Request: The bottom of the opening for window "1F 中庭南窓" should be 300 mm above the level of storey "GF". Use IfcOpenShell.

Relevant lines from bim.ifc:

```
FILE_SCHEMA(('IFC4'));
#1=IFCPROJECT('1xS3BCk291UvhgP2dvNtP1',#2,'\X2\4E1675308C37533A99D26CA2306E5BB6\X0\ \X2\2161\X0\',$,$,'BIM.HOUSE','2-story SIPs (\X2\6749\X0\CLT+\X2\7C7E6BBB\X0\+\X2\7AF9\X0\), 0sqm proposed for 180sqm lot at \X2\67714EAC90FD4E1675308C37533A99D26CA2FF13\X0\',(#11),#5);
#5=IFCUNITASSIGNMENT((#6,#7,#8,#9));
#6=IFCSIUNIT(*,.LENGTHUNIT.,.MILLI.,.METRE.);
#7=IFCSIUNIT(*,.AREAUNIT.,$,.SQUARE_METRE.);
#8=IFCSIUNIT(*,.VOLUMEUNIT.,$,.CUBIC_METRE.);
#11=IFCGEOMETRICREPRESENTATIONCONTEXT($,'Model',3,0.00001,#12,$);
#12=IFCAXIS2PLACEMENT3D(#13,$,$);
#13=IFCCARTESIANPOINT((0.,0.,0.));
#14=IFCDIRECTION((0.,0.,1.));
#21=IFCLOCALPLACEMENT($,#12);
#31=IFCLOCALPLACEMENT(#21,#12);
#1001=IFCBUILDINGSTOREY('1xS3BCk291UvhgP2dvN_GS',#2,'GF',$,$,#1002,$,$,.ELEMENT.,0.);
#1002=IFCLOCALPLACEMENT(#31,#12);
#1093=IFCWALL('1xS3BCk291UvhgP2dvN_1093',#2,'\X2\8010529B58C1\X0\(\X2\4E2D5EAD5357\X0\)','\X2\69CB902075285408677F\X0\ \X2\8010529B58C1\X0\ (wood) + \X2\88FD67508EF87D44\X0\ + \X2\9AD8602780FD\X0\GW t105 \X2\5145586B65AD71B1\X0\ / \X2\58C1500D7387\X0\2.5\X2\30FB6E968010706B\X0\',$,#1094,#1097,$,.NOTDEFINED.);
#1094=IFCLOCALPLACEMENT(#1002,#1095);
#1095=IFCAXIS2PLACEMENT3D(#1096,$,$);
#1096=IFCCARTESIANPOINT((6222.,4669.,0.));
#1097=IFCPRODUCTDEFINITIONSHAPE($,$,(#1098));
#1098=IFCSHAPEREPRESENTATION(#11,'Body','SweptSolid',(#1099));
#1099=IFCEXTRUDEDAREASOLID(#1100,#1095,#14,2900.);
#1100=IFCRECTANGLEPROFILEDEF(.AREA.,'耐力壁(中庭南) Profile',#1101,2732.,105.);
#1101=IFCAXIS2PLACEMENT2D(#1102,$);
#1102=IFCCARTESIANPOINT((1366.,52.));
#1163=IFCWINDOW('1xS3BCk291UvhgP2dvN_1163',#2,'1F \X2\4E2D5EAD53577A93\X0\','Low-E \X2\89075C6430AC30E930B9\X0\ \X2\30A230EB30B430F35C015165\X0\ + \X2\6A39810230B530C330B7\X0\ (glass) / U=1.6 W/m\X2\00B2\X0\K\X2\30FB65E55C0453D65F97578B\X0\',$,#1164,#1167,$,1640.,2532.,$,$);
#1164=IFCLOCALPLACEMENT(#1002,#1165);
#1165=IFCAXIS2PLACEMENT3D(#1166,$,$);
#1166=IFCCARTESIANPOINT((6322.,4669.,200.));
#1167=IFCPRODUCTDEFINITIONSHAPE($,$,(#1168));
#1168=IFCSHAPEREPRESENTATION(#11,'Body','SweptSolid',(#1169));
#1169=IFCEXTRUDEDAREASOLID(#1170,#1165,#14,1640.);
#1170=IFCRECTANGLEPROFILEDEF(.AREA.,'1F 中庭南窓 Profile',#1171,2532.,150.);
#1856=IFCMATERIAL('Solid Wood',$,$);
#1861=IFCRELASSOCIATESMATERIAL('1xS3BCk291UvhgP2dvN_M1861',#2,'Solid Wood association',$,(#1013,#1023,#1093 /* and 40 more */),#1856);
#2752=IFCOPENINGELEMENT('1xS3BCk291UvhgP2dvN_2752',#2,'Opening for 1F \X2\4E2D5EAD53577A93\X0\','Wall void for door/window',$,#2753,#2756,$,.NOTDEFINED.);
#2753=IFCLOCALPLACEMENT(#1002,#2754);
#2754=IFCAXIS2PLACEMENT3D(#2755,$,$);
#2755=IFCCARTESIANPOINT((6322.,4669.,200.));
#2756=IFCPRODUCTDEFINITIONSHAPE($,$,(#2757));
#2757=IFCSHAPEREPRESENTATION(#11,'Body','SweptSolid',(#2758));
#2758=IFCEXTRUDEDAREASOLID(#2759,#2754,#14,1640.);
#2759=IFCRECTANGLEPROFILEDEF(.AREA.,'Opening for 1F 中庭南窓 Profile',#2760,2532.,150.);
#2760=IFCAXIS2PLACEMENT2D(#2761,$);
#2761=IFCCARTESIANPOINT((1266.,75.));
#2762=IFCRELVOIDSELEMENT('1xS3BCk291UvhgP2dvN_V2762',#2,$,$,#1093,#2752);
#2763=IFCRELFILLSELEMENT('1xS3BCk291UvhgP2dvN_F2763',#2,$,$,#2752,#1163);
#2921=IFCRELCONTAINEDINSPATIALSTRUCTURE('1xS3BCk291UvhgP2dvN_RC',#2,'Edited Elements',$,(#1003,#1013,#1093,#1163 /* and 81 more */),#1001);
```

```python
import numpy as np
import ifcopenshell
import ifcopenshell.api.geometry
import ifcopenshell.geom
import ifcopenshell.util.element
import ifcopenshell.util.placement
import ifcopenshell.util.shape
import ifcopenshell.util.unit

model = ifcopenshell.open("bim.ifc")
unit_scale = ifcopenshell.util.unit.calculate_unit_scale(model)

window = model.by_guid("1xS3BCk291UvhgP2dvN_1163")
opening = window.FillsVoids[0].RelatingOpeningElement
storey = ifcopenshell.util.element.get_container(window, ifc_class="IfcBuildingStorey")
level = ifcopenshell.util.placement.get_local_placement(storey.ObjectPlacement)[2, 3]

# The opening's origin need not be at the sill, so measure its lowest point.
shape = ifcopenshell.geom.create_shape(ifcopenshell.geom.settings(), opening)
bottom = ifcopenshell.util.shape.get_shape_bottom_elevation(shape, shape.geometry) / unit_scale
dz = level + 0.3 / unit_scale - bottom

shift = np.array([0.0, 0.0, dz])
# The window is not placed relative to its opening, so move both.
for product in (opening, window):
    matrix = ifcopenshell.util.placement.get_local_placement(product.ObjectPlacement)
    matrix[:3, 3] += shift
    ifcopenshell.api.geometry.edit_object_placement(model, product=product, matrix=matrix, is_si=False)

print(f"moved by {dz * unit_scale:+.3f} m")

model.write("bim-out.ifc")
```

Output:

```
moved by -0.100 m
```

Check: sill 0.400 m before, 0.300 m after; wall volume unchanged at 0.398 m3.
